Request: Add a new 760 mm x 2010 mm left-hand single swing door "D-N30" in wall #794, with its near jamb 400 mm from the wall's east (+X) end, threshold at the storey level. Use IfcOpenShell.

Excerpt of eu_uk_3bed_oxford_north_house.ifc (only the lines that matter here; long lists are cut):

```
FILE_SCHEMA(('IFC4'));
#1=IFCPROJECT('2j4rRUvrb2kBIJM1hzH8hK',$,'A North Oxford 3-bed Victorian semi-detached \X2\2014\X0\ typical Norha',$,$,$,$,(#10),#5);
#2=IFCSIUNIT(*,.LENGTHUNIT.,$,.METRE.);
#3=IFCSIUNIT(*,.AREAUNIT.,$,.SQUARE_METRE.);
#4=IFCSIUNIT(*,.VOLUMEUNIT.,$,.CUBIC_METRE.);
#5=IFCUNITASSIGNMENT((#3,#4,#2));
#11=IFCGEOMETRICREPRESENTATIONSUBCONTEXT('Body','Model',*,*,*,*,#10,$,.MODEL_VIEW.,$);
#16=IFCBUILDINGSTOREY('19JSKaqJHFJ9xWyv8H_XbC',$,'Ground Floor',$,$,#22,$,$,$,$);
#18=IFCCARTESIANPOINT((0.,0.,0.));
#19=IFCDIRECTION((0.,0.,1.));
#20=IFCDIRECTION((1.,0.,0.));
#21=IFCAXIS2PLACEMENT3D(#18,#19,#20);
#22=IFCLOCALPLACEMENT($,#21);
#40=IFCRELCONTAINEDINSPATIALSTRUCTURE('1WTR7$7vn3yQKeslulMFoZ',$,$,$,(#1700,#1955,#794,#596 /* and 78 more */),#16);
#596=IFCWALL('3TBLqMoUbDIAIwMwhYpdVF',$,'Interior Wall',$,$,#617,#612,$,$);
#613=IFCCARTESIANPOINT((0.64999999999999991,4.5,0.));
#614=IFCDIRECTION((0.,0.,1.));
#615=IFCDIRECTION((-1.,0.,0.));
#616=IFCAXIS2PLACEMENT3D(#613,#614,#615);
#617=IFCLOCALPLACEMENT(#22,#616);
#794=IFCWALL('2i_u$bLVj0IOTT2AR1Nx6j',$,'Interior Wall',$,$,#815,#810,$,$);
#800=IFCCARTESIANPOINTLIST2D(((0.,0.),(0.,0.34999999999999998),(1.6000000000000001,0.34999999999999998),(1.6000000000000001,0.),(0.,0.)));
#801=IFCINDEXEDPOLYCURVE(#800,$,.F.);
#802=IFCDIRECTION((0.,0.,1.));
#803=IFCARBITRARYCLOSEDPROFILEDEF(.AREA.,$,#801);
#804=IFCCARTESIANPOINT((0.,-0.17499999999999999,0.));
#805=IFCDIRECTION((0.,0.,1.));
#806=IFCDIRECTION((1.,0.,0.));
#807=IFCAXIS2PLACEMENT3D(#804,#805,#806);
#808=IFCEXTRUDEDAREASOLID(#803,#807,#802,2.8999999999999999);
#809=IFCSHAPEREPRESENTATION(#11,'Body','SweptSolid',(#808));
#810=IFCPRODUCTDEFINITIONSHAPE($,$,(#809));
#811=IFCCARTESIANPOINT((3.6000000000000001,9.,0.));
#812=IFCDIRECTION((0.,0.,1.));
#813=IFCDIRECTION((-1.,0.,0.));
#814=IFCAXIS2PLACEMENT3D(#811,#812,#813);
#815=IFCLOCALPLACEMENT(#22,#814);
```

```python
import numpy as np
import ifcopenshell
import ifcopenshell.api.feature
import ifcopenshell.api.geometry
import ifcopenshell.api.root
import ifcopenshell.api.spatial
import ifcopenshell.geom
import ifcopenshell.util.element
import ifcopenshell.util.placement
import ifcopenshell.util.representation
import ifcopenshell.util.shape
import ifcopenshell.util.unit

model = ifcopenshell.open("eu_uk_3bed_oxford_north_house.ifc")
unit_scale = ifcopenshell.util.unit.calculate_unit_scale(model)
settings = ifcopenshell.geom.settings()


def volume(element):
    """Net volume in cubic metres, openings subtracted."""
    shape = ifcopenshell.geom.create_shape(settings, element)
    return ifcopenshell.util.shape.get_volume(shape.geometry)


wall = model.by_guid("2i_u$bLVj0IOTT2AR1Nx6j")
storey = ifcopenshell.util.element.get_container(wall, ifc_class="IfcBuildingStorey")
context = ifcopenshell.util.representation.get_context(model, "Model", "Body", "MODEL_VIEW")
before = volume(wall)

width, height, from_end, sill = 0.76, 2.01, 0.4, 0.0  # metres

# The wall runs along its own X axis, and the end named is its -X end.
wall_shape = ifcopenshell.geom.create_shape(settings, wall)
x, y, z = ifcopenshell.util.shape.get_vertices(wall_shape.geometry).T
start = x.min() + from_end
face, thickness = float(y.min()), float(y.max() - y.min())
wall_matrix = ifcopenshell.util.placement.get_local_placement(wall.ObjectPlacement)
level = ifcopenshell.util.placement.get_local_placement(storey.ObjectPlacement)[2, 3]


def in_wall(x, y):
    """Placement at x, y metres in the wall's axes, at sill height."""
    matrix = wall_matrix.copy()
    matrix[:, 3] = wall_matrix @ np.array([x / unit_scale, y / unit_scale, 0.0, 1.0])
    matrix[2, 3] = level + sill / unit_scale
    return matrix


# Opening: a box that overshoots both wall faces by 50 mm.
opening = ifcopenshell.api.root.create_entity(model, ifc_class="IfcOpeningElement", predefined_type="OPENING")
box = ifcopenshell.api.geometry.add_wall_representation(
    model, context=context, length=width, height=height, thickness=thickness + 0.1
)
ifcopenshell.api.geometry.assign_representation(model, product=opening, representation=box)
ifcopenshell.api.geometry.edit_object_placement(model, product=opening, matrix=in_wall(start, face - 0.05), is_si=False)
ifcopenshell.api.feature.add_feature(model, feature=opening, element=wall)

door = ifcopenshell.api.root.create_entity(model, ifc_class="IfcDoor", name="D-N30", predefined_type="DOOR")
door.OverallWidth, door.OverallHeight = width / unit_scale, height / unit_scale
door.OperationType = "SINGLE_SWING_LEFT"
body = ifcopenshell.api.geometry.add_door_representation(
    model,
    context=context,
    overall_width=door.OverallWidth,
    overall_height=door.OverallHeight,
    operation_type="SINGLE_SWING_LEFT",
    lining_properties={"LiningDepth": thickness / unit_scale, "ThresholdDepth": thickness / unit_scale},
)
ifcopenshell.api.geometry.assign_representation(model, product=door, representation=body)
ifcopenshell.api.spatial.assign_container(model, products=[door], relating_structure=storey)
ifcopenshell.api.feature.add_filling(model, opening=opening, element=door)

# The lining spans the wall, so the door starts at the wall face.
ifcopenshell.api.geometry.edit_object_placement(model, product=door, matrix=in_wall(start, face), is_si=False)

after = volume(wall)

print(f"wall volume {before:.3f} -> {after:.3f} m3")

model.write("eu_uk_3bed_oxford_north_house-out.ifc")
```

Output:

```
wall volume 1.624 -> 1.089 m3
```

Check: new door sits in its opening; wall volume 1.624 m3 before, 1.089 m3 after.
